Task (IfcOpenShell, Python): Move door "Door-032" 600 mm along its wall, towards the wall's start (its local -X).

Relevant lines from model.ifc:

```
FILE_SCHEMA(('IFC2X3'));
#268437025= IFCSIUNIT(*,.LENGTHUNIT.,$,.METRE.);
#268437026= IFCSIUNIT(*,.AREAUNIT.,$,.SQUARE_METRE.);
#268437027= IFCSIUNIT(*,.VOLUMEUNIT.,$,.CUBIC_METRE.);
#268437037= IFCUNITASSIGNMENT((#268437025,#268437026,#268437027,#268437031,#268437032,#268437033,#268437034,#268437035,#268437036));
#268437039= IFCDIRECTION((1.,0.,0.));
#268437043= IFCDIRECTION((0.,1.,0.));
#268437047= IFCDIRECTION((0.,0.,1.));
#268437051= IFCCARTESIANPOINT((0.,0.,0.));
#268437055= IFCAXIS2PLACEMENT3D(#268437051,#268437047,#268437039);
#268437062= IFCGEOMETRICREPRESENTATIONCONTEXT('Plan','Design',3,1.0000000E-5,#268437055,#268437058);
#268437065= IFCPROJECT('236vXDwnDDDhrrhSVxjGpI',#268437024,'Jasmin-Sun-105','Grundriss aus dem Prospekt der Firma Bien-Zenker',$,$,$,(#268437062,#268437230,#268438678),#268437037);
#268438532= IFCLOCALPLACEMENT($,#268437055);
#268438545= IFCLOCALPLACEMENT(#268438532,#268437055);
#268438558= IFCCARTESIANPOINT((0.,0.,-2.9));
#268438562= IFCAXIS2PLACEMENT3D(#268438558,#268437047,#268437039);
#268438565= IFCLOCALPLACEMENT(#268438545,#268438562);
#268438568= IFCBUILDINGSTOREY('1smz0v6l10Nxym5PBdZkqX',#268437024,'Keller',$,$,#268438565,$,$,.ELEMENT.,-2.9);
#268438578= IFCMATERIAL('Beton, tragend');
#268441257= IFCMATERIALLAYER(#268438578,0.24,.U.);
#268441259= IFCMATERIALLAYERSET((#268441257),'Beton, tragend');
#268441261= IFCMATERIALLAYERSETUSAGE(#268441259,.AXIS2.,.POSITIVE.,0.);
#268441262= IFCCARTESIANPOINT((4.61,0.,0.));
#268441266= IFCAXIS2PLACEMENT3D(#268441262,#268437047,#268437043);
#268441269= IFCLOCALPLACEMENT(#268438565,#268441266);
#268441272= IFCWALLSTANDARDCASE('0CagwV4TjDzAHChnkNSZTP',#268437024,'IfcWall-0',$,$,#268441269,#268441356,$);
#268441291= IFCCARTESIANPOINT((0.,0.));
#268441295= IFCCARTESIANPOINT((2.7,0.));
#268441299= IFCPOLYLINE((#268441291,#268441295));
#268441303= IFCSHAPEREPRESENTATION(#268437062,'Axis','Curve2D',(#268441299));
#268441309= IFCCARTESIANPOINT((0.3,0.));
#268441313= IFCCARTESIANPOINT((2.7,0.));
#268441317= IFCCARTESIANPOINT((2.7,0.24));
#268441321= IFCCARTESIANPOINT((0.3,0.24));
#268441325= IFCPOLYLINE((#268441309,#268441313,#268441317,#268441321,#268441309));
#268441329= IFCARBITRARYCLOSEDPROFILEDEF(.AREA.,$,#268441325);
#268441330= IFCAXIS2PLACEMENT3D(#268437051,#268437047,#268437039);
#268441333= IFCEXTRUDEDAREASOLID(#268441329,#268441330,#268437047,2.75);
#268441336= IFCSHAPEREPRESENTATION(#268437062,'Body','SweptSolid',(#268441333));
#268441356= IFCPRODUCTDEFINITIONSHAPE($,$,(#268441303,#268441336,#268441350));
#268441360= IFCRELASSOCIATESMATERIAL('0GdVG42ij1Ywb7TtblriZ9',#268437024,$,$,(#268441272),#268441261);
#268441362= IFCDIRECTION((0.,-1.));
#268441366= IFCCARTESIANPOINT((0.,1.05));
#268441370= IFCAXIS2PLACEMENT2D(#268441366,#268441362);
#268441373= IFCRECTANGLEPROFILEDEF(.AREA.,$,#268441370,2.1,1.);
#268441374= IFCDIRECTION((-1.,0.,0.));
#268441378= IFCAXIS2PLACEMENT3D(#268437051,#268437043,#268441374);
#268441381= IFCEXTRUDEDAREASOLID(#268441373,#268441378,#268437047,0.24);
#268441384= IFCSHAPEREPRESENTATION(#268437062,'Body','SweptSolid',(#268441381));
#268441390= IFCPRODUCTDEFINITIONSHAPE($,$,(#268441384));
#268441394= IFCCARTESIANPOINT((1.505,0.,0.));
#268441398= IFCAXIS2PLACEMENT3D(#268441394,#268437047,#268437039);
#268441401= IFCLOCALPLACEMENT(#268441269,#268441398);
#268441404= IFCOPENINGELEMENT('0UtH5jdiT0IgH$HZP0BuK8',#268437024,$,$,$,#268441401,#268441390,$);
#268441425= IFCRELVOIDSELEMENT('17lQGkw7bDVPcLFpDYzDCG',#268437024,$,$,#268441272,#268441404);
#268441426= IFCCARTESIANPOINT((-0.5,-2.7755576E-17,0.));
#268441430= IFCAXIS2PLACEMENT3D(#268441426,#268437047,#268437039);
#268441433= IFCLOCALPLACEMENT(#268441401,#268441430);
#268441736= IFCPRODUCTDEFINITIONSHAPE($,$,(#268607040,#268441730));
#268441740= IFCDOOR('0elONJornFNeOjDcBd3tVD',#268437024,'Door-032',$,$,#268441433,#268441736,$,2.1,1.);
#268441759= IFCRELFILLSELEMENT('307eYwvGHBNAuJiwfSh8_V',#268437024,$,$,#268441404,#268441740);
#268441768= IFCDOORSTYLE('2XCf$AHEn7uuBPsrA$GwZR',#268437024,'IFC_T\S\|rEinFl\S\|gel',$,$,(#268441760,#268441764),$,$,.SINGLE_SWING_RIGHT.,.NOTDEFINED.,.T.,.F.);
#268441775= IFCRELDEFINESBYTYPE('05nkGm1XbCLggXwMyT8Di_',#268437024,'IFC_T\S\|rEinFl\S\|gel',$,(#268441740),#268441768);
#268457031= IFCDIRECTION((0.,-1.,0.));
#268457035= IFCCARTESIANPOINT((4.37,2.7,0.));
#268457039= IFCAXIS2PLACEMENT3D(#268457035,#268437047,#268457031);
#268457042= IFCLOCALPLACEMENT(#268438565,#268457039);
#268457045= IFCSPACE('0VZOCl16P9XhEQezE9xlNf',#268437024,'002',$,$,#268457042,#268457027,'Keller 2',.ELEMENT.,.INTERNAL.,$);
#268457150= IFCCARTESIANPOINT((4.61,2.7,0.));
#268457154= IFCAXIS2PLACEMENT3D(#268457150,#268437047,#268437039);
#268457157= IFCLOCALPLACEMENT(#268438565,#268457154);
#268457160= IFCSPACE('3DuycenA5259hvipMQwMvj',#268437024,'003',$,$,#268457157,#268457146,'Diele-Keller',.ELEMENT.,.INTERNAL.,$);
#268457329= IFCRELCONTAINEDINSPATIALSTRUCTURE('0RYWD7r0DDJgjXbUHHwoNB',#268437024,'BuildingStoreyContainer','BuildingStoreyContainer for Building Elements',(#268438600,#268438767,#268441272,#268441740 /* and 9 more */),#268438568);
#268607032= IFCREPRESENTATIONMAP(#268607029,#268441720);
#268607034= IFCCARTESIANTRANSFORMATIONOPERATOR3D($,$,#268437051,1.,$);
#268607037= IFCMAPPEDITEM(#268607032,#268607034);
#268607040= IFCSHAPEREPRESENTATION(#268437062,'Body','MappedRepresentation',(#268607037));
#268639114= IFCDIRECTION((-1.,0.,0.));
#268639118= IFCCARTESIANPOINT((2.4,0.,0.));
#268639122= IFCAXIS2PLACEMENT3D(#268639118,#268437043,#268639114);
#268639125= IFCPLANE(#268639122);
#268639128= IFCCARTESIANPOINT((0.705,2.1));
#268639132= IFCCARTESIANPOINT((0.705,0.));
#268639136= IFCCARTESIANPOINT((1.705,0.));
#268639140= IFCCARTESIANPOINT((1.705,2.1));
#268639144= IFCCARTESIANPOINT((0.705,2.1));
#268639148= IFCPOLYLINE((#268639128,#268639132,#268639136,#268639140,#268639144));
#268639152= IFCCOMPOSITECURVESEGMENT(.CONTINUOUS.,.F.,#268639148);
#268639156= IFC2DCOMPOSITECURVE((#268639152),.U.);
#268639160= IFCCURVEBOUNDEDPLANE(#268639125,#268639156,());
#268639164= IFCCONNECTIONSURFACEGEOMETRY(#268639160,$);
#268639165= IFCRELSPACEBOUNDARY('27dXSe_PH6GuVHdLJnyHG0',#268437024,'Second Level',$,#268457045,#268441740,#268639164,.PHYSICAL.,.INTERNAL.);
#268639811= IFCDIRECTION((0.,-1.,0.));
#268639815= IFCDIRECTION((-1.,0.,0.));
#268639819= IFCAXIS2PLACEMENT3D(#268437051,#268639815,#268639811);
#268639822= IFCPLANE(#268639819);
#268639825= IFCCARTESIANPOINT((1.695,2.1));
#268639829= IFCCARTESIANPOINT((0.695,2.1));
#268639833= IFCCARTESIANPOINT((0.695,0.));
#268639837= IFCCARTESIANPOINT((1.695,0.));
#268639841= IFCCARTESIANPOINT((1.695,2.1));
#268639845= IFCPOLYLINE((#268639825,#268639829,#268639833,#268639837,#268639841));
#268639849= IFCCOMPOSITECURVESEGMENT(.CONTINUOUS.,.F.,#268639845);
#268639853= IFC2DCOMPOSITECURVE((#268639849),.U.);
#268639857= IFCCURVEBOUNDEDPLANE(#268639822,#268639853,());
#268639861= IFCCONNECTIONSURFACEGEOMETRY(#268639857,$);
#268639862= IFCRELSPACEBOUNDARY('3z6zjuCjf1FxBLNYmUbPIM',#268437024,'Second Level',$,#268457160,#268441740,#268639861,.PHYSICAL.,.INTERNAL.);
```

```python
import numpy as np
import ifcopenshell
import ifcopenshell.api.geometry
import ifcopenshell.util.placement
import ifcopenshell.util.unit

model = ifcopenshell.open("model.ifc")
unit_scale = ifcopenshell.util.unit.calculate_unit_scale(model)

door = model.by_guid("0elONJornFNeOjDcBd3tVD")
opening = door.FillsVoids[0].RelatingOpeningElement
wall = opening.VoidsElements[0].RelatingBuildingElement

wall_matrix = ifcopenshell.util.placement.get_local_placement(wall.ObjectPlacement)
shift = wall_matrix[:3, 0] * -0.6 / unit_scale
before = ifcopenshell.util.placement.get_local_placement(door.ObjectPlacement)[:3, 3].copy()

# The door is placed relative to its opening, so it follows when the opening moves.
matrix = ifcopenshell.util.placement.get_local_placement(opening.ObjectPlacement)
matrix[:3, 3] += shift
ifcopenshell.api.geometry.edit_object_placement(
    model, product=opening, matrix=matrix, is_si=False, should_transform_children=True
)

# Space boundary surfaces are stored in each space's coordinates; move them too.
for rel in door.ProvidesBoundaries:
    if not rel.ConnectionGeometry:
        continue
    surface = rel.ConnectionGeometry.SurfaceOnRelatingElement.BasisSurface
    space_matrix = ifcopenshell.util.placement.get_local_placement(rel.RelatingSpace.ObjectPlacement)
    point = np.array(surface.Position.Location.Coordinates) + space_matrix[:3, :3].T @ shift
    surface.Position = model.createIfcAxis2Placement3D(
        model.createIfcCartesianPoint(point.tolist()), surface.Position.Axis, surface.Position.RefDirection
    )

after = ifcopenshell.util.placement.get_local_placement(door.ObjectPlacement)[:3, 3]
print("door moved by", (after - before).round(3) + 0.0)

model.write("model-out.ifc")
```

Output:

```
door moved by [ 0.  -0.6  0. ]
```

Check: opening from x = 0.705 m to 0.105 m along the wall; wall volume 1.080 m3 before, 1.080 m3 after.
